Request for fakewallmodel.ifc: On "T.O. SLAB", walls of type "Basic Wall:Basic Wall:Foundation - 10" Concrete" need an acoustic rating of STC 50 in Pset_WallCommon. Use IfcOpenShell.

First a look at what the model holds.

```python
import ifcopenshell
import ifcopenshell.util.element

model = ifcopenshell.open("fakewallmodel.ifc")
print(model.schema)
storey = next(s for s in model.by_type("IfcBuildingStorey") if s.Name == "T.O. SLAB")
walls = [e for e in ifcopenshell.util.element.get_decomposition(storey) if e.is_a("IfcWall")]
seen = {}
for e in walls:
    element_type = ifcopenshell.util.element.get_type(e)
    key = (element_type.Name if element_type != e and element_type else None, ifcopenshell.util.element.get_pset(e, "Pset_WallCommon", "AcousticRating"))
    seen[key] = seen.get(key, 0) + 1
for (name, value), count in sorted(seen.items(), key=str):
    print(count, "x", name, "|", value)
```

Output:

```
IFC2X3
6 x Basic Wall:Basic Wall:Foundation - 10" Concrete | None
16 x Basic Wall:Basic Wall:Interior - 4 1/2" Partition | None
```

```python
import ifcopenshell
import ifcopenshell.api.pset
import ifcopenshell.util.element

model = ifcopenshell.open("fakewallmodel.ifc")

storey = next(s for s in model.by_type("IfcBuildingStorey") if s.Name == "T.O. SLAB")
walls = [e for e in ifcopenshell.util.element.get_decomposition(storey) if e.is_a("IfcWall")]

count = 0
for e in walls:
    element_type = ifcopenshell.util.element.get_type(e)
    if element_type in (None, e) or element_type.Name != 'Basic Wall:Basic Wall:Foundation - 10" Concrete':
        continue
    # add_pset returns the element's existing set when there is one.
    pset = ifcopenshell.api.pset.add_pset(model, product=e, name="Pset_WallCommon")
    ifcopenshell.api.pset.edit_pset(model, pset=pset, properties={"AcousticRating": "STC 50"})
    count += 1

print(count, "walls updated")

model.write("fakewallmodel_rev.ifc")
```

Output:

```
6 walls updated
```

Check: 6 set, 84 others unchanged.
